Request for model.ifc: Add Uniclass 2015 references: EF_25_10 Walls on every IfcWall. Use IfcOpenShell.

First a look at what the model holds.

```python
import ifcopenshell

model = ifcopenshell.open("model.ifc")
print(model.schema)
print("classifications:", [c.Name for c in model.by_type("IfcClassification")])
for ifc_class in ("IfcDoor", "IfcRoof", "IfcStair", "IfcWall", "IfcWindow"):
    print(ifc_class, len(model.by_type(ifc_class)))
```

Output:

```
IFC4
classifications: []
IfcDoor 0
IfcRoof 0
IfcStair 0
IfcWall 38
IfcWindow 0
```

```python
import ifcopenshell
import ifcopenshell.api.classification

model = ifcopenshell.open("model.ifc")

system = ifcopenshell.api.classification.add_classification(model, classification="Uniclass 2015")

codes = {
    "IfcWall": ("EF_25_10", "Walls"),
}
for ifc_class, (code, name) in codes.items():
    products = model.by_type(ifc_class)
    ifcopenshell.api.classification.add_reference(
        model, products=products, classification=system, identification=code, name=name
    )
    print(code, len(products))

model.write("model_edited.ifc")
```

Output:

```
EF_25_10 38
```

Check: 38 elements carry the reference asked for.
